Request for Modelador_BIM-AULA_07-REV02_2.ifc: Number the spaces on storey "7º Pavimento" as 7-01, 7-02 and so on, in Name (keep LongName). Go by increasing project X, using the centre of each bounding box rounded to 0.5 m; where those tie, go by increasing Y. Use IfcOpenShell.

First a look at what the model holds.

```python
import ifcopenshell
import ifcopenshell.util.element
import ifcopenshell.util.placement

model = ifcopenshell.open("Modelador_BIM-AULA_07-REV02_2.ifc")
print(model.schema)
storey = next(s for s in model.by_type("IfcBuildingStorey") if s.Name == "7º Pavimento")
spaces = [e for e in ifcopenshell.util.element.get_decomposition(storey) if e.is_a("IfcSpace")]
for e in sorted(spaces, key=lambda e: e.id()):
    origin = ifcopenshell.util.placement.get_local_placement(e.ObjectPlacement)[:3, 3]
    print(e.id(), e.Name, e.LongName, origin.round(2) + 0.0, sep=" | ")
```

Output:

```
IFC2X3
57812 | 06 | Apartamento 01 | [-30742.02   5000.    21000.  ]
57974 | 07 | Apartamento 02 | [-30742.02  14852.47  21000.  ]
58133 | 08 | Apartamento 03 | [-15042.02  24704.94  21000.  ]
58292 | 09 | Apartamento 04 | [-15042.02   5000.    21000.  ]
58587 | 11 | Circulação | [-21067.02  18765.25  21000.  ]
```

```python
import ifcopenshell
import ifcopenshell.geom
import ifcopenshell.util.element
import ifcopenshell.util.shape

model = ifcopenshell.open("Modelador_BIM-AULA_07-REV02_2.ifc")
settings = ifcopenshell.geom.settings()
settings.set("use-world-coords", True)


def centre(element):
    shape = ifcopenshell.geom.create_shape(settings, element)
    return ifcopenshell.util.shape.get_bbox_centroid(shape.geometry)


storey = next(s for s in model.by_type("IfcBuildingStorey") if s.Name == "7º Pavimento")
spaces = [e for e in ifcopenshell.util.element.get_decomposition(storey) if e.is_a("IfcSpace")]

# Insertion points can sit at a corner or the storey origin, so sort by the geometry (in metres).
centres = {e: centre(e) for e in spaces}
spaces.sort(key=lambda e: (round(centres[e][0] / 0.5), centres[e][1]))

for i, e in enumerate(spaces, start=1):
    number = f"7-{i:02d}"
    e.Name = number
    print(e.id(), number)

model.write("Modelador_BIM-AULA_07-REV02_2_edited.ifc")
```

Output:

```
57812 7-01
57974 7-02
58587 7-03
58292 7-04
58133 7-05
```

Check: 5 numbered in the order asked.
